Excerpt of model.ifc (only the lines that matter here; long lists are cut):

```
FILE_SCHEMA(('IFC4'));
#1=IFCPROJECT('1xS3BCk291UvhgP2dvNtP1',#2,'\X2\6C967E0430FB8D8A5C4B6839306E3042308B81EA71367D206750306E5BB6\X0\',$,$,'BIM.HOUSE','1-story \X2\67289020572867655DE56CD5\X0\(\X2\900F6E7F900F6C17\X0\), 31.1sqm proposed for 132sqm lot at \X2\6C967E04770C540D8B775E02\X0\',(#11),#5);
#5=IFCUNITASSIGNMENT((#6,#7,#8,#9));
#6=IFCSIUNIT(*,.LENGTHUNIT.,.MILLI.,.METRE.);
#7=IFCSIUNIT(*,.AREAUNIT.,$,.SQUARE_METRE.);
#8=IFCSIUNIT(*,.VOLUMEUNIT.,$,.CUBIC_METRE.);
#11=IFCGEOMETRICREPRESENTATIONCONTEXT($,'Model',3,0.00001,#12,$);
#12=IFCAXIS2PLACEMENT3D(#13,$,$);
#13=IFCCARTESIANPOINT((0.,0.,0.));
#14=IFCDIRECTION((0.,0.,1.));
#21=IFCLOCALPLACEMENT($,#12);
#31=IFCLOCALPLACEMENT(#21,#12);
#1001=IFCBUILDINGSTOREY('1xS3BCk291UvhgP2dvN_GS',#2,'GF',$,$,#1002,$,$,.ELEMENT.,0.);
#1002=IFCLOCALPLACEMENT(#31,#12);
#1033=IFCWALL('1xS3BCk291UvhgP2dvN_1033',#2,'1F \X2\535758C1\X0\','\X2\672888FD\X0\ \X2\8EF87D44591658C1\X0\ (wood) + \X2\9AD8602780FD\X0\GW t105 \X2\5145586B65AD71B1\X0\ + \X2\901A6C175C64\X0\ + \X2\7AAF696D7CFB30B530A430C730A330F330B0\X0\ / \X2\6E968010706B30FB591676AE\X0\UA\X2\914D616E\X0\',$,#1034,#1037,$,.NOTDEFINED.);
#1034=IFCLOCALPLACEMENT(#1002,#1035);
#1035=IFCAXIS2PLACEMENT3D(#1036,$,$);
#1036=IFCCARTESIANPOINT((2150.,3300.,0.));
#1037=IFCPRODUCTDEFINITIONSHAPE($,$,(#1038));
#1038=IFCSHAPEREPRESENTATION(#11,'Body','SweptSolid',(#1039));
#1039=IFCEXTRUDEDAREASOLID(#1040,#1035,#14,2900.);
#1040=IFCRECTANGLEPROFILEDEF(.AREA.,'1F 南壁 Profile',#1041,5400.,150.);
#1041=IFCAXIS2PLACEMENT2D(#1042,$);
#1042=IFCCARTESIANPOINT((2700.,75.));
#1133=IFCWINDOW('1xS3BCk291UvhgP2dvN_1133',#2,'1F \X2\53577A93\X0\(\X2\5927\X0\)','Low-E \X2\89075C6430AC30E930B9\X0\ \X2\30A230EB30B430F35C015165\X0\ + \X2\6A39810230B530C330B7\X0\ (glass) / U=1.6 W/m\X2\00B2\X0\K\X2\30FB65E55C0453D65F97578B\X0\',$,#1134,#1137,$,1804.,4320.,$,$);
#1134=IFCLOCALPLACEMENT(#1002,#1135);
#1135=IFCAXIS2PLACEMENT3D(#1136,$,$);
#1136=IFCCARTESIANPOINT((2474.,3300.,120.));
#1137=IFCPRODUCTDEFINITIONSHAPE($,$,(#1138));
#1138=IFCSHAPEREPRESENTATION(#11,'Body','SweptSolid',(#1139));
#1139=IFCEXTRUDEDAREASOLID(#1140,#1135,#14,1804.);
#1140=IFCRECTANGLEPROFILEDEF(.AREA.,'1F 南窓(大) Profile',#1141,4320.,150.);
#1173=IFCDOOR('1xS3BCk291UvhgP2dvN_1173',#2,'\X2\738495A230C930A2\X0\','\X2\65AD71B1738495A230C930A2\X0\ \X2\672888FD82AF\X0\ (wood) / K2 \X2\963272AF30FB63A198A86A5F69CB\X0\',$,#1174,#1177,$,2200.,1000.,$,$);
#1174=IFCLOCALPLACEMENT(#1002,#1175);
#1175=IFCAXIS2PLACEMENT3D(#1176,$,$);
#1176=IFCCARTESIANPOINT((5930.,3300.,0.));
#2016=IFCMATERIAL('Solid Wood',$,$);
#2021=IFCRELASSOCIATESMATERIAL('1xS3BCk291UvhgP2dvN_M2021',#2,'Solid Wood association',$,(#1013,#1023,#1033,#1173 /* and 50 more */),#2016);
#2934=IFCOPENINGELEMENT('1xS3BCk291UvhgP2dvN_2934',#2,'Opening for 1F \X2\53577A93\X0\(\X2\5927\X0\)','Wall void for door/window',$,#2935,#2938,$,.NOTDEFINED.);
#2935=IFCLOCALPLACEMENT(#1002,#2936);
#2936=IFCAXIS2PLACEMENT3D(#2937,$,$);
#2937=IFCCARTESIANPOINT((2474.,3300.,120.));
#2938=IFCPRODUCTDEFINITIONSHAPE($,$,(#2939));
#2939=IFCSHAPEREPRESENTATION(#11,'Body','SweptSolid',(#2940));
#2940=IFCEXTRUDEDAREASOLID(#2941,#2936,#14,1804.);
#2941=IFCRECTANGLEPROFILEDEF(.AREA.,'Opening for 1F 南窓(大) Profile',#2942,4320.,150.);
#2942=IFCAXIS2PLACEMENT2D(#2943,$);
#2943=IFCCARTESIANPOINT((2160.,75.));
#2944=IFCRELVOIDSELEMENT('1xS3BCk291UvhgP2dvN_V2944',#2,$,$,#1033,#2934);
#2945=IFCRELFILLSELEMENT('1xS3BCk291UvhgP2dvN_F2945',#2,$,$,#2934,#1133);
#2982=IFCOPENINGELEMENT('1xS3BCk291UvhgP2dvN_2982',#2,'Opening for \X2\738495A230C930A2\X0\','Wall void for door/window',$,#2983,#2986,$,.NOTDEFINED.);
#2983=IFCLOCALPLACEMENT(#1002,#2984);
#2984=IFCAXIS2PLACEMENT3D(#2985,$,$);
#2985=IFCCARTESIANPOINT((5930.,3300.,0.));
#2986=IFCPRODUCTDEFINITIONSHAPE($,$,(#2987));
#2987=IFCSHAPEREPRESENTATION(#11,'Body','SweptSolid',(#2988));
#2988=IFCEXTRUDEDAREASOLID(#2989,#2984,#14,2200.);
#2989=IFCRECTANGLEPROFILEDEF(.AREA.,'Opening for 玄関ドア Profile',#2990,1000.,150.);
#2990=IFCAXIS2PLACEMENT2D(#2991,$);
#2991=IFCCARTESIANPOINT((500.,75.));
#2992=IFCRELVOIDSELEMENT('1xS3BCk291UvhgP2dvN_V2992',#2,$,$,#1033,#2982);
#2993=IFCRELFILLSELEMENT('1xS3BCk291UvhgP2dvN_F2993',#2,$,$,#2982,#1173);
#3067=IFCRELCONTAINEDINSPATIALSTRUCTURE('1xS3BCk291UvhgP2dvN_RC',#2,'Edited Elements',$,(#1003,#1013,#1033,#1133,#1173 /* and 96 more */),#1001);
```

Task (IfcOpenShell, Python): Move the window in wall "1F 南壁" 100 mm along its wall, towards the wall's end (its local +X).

```python
import ifcopenshell
import ifcopenshell.api.geometry
import ifcopenshell.util.placement
import ifcopenshell.util.unit

model = ifcopenshell.open("model.ifc")
unit_scale = ifcopenshell.util.unit.calculate_unit_scale(model)

window = model.by_guid("1xS3BCk291UvhgP2dvN_1133")
opening = window.FillsVoids[0].RelatingOpeningElement
wall = opening.VoidsElements[0].RelatingBuildingElement

wall_matrix = ifcopenshell.util.placement.get_local_placement(wall.ObjectPlacement)
shift = wall_matrix[:3, 0] * 0.1 / unit_scale
before = ifcopenshell.util.placement.get_local_placement(window.ObjectPlacement)[:3, 3].copy()

# The window is not placed relative to its opening, so move both.
for product in (opening, window):
    matrix = ifcopenshell.util.placement.get_local_placement(product.ObjectPlacement)
    matrix[:3, 3] += shift
    ifcopenshell.api.geometry.edit_object_placement(model, product=product, matrix=matrix, is_si=False)

after = ifcopenshell.util.placement.get_local_placement(window.ObjectPlacement)[:3, 3]
print("window moved by", (after - before).round(3) + 0.0)

model.write("model-out.ifc")
```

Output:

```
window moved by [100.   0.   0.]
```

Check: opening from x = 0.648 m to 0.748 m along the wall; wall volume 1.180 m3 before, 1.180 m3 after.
